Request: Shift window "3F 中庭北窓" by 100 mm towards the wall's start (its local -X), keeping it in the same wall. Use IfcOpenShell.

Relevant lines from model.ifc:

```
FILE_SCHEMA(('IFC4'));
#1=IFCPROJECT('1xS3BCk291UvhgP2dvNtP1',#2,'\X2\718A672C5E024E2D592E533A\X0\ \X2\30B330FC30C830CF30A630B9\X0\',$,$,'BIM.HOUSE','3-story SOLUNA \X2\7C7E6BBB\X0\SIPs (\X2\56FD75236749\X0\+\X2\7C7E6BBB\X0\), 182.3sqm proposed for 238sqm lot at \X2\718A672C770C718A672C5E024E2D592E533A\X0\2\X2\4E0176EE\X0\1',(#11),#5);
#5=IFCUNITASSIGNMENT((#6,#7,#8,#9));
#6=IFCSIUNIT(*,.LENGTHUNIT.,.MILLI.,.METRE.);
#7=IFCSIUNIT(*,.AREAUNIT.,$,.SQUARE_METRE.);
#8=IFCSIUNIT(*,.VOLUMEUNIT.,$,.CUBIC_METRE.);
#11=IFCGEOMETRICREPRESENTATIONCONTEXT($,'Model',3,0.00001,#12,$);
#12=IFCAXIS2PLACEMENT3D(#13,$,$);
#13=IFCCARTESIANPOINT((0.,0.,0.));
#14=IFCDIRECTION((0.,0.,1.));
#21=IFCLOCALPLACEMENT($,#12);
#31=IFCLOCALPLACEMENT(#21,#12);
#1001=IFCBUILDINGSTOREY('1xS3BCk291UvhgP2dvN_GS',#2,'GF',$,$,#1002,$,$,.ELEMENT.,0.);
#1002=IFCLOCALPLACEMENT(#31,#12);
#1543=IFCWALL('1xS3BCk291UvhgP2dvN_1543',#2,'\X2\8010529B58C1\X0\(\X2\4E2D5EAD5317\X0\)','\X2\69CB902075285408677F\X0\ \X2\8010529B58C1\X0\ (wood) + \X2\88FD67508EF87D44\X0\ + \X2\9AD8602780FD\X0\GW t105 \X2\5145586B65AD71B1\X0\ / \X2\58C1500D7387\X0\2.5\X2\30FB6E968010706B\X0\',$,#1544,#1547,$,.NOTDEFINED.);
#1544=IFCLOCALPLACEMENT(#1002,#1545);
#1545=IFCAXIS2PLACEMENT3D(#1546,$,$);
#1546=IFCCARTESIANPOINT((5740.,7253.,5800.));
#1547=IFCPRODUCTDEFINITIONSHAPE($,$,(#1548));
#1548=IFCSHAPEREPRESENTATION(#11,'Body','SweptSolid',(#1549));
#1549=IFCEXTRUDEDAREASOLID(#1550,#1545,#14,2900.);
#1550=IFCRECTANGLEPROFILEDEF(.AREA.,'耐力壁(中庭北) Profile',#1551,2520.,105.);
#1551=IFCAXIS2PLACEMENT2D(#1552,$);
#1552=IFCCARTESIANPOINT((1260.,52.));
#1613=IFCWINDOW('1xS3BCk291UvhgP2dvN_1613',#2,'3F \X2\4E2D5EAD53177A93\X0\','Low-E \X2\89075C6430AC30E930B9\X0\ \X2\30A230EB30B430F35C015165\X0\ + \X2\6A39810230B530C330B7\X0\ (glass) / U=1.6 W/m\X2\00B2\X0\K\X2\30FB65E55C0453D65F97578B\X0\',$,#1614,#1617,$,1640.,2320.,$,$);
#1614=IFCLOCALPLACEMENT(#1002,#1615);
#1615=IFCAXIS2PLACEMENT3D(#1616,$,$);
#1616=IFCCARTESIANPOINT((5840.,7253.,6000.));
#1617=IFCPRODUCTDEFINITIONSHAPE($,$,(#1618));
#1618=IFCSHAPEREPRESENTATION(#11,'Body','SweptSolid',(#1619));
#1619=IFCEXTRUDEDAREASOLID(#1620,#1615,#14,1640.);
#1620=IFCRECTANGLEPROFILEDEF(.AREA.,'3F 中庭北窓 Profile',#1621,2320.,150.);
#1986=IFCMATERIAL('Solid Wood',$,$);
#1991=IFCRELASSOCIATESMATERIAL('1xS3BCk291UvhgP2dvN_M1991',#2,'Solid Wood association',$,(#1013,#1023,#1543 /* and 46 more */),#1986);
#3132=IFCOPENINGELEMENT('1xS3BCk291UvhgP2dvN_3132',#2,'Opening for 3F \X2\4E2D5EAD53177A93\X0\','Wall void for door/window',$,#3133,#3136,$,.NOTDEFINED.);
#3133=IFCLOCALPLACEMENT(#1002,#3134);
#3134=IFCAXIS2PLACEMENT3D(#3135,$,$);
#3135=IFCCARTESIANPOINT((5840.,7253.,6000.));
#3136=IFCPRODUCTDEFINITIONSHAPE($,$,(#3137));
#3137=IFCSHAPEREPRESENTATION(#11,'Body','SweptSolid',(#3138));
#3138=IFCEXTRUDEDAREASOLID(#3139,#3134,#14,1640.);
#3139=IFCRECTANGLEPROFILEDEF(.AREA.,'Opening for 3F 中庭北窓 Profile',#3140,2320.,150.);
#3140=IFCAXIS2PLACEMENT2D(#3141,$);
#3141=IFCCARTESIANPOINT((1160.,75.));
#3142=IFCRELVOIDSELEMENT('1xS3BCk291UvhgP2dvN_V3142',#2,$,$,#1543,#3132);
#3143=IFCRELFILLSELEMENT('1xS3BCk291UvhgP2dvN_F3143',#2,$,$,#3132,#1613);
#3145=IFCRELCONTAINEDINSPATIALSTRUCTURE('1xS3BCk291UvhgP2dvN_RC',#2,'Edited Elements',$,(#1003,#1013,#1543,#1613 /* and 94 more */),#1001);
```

```python
import ifcopenshell
import ifcopenshell.api.geometry
import ifcopenshell.util.placement
import ifcopenshell.util.unit

model = ifcopenshell.open("model.ifc")
unit_scale = ifcopenshell.util.unit.calculate_unit_scale(model)

window = model.by_guid("1xS3BCk291UvhgP2dvN_1613")
opening = window.FillsVoids[0].RelatingOpeningElement
wall = opening.VoidsElements[0].RelatingBuildingElement

wall_matrix = ifcopenshell.util.placement.get_local_placement(wall.ObjectPlacement)
shift = wall_matrix[:3, 0] * -0.1 / unit_scale
before = ifcopenshell.util.placement.get_local_placement(window.ObjectPlacement)[:3, 3].copy()

# The window is not placed relative to its opening, so move both.
for product in (opening, window):
    matrix = ifcopenshell.util.placement.get_local_placement(product.ObjectPlacement)
    matrix[:3, 3] += shift
    ifcopenshell.api.geometry.edit_object_placement(model, product=product, matrix=matrix, is_si=False)

after = ifcopenshell.util.placement.get_local_placement(window.ObjectPlacement)[:3, 3]
print("window moved by", (after - before).round(3) + 0.0)

model.write("model_updated.ifc")
```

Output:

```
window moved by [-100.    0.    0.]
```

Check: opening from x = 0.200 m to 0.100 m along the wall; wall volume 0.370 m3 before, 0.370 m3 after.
